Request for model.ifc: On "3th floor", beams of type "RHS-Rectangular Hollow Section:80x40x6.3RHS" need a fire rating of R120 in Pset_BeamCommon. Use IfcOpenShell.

First a look at what the model holds.

```python
import ifcopenshell
import ifcopenshell.util.element

model = ifcopenshell.open("model.ifc")
print(model.schema)
storey = next(s for s in model.by_type("IfcBuildingStorey") if s.Name == "3th floor")
beams = [e for e in ifcopenshell.util.element.get_decomposition(storey) if e.is_a("IfcBeam")]
seen = {}
for e in beams:
    element_type = ifcopenshell.util.element.get_type(e)
    key = (element_type.Name if element_type != e and element_type else None, ifcopenshell.util.element.get_pset(e, "Pset_BeamCommon", "FireRating"))
    seen[key] = seen.get(key, 0) + 1
for (name, value), count in sorted(seen.items(), key=str):
    print(count, "x", name, "|", value)
```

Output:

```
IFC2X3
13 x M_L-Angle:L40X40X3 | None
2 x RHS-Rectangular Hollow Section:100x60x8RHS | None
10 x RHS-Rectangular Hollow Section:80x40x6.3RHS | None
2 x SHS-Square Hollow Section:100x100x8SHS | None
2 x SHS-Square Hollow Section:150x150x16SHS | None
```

```python
import ifcopenshell
import ifcopenshell.api.pset
import ifcopenshell.util.element

model = ifcopenshell.open("model.ifc")

storey = next(s for s in model.by_type("IfcBuildingStorey") if s.Name == "3th floor")
beams = [e for e in ifcopenshell.util.element.get_decomposition(storey) if e.is_a("IfcBeam")]

count = 0
for e in beams:
    element_type = ifcopenshell.util.element.get_type(e)
    if element_type in (None, e) or element_type.Name != "RHS-Rectangular Hollow Section:80x40x6.3RHS":
        continue
    # add_pset returns the element's existing set when there is one.
    pset = ifcopenshell.api.pset.add_pset(model, product=e, name="Pset_BeamCommon")
    ifcopenshell.api.pset.edit_pset(model, pset=pset, properties={"FireRating": "R120"})
    count += 1

print(count, "beams updated")

model.write("model_rev.ifc")
```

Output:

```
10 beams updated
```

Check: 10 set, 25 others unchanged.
